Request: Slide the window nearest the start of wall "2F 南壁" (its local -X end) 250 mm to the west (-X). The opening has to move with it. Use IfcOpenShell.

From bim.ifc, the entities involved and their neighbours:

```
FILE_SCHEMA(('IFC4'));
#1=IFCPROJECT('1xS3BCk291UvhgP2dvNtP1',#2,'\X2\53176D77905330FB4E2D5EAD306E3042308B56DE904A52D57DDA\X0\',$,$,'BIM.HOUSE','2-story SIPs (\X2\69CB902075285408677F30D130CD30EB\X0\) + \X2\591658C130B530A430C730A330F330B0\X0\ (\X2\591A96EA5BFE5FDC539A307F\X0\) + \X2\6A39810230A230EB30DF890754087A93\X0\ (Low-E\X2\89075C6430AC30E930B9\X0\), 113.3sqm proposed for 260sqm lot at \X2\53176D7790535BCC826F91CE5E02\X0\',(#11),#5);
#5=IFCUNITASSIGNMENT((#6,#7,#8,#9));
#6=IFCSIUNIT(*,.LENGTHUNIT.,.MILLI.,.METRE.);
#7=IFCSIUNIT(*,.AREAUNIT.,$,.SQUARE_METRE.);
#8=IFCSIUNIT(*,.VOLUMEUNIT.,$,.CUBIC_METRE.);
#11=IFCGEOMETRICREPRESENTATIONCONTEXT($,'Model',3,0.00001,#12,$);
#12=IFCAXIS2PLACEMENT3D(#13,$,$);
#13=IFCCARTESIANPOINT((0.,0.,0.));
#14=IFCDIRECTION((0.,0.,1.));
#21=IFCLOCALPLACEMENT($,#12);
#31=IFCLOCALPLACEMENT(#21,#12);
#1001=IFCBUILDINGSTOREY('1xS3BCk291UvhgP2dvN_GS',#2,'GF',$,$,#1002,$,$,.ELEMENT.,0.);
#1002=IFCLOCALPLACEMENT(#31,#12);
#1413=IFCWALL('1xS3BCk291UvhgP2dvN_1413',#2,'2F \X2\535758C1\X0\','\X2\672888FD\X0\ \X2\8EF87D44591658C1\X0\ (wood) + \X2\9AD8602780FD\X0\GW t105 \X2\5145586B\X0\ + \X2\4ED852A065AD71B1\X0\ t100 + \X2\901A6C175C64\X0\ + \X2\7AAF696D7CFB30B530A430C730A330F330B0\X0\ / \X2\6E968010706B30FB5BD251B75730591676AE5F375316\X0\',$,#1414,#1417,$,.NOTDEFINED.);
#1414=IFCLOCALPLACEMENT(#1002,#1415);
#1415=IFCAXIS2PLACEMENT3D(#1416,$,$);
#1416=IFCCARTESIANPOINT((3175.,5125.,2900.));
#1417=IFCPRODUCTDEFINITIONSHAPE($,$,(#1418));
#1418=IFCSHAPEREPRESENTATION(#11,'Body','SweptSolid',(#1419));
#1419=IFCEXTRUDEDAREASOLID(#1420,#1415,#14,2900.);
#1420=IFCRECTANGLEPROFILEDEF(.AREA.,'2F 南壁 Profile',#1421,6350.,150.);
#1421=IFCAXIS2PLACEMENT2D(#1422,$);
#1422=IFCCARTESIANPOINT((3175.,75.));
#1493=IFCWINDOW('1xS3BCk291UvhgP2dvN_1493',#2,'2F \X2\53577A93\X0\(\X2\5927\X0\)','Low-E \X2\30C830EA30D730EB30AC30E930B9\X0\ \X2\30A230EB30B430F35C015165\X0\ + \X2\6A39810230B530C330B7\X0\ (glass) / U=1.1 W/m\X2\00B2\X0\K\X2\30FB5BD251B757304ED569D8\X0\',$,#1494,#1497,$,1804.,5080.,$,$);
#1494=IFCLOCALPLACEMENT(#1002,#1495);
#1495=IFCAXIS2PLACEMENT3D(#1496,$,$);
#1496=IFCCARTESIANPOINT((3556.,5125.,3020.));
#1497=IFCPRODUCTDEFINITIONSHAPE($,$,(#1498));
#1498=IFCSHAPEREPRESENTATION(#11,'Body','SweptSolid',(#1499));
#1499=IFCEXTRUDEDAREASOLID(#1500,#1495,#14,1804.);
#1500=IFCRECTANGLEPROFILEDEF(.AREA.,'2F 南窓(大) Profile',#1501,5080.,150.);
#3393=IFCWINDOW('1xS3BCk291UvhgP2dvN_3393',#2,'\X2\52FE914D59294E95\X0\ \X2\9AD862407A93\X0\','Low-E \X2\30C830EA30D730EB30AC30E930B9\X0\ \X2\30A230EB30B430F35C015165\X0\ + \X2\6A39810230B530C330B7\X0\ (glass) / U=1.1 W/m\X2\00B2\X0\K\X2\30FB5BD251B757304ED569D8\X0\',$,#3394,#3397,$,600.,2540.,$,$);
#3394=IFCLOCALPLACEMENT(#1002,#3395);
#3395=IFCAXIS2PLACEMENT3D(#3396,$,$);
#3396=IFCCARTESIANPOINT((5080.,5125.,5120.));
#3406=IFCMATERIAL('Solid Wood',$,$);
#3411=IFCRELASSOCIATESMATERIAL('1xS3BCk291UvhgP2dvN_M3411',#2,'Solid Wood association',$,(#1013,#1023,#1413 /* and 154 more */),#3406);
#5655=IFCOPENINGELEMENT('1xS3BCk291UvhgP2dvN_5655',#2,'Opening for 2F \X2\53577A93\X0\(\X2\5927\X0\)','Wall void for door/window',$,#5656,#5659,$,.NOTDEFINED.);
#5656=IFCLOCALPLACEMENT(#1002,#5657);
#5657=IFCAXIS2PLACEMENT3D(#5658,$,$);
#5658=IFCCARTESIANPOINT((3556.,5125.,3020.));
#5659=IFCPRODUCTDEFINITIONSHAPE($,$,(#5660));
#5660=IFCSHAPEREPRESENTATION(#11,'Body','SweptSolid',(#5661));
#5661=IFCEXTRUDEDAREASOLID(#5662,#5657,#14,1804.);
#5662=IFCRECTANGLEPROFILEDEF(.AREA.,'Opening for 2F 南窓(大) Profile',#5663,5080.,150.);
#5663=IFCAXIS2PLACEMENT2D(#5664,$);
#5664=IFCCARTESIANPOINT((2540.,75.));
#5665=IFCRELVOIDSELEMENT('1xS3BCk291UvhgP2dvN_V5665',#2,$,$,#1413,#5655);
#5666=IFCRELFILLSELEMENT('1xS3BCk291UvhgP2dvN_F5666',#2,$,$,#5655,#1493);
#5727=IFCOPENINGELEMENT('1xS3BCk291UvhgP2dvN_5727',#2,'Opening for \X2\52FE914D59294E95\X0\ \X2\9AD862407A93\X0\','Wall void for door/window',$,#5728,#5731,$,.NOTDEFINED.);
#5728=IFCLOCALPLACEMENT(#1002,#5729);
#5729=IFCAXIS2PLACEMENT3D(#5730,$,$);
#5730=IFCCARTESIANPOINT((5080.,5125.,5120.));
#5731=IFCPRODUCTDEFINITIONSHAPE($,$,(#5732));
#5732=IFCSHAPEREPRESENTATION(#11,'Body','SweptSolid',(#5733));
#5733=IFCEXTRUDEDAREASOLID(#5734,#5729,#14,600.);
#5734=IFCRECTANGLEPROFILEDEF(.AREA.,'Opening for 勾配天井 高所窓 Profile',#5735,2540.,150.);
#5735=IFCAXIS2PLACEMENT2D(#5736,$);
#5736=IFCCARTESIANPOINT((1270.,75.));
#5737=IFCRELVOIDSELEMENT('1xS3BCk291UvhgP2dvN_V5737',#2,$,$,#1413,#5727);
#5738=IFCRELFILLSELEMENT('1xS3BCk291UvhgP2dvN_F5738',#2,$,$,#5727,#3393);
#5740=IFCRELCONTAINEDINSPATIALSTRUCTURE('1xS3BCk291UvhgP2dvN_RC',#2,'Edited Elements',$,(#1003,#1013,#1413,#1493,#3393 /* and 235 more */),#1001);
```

```python
import ifcopenshell
import ifcopenshell.api.geometry
import ifcopenshell.util.placement
import ifcopenshell.util.unit

model = ifcopenshell.open("bim.ifc")
unit_scale = ifcopenshell.util.unit.calculate_unit_scale(model)

window = model.by_guid("1xS3BCk291UvhgP2dvN_1493")
opening = window.FillsVoids[0].RelatingOpeningElement
wall = opening.VoidsElements[0].RelatingBuildingElement

wall_matrix = ifcopenshell.util.placement.get_local_placement(wall.ObjectPlacement)
shift = wall_matrix[:3, 0] * -0.25 / unit_scale
before = ifcopenshell.util.placement.get_local_placement(window.ObjectPlacement)[:3, 3].copy()

# The window is not placed relative to its opening, so move both.
for product in (opening, window):
    matrix = ifcopenshell.util.placement.get_local_placement(product.ObjectPlacement)
    matrix[:3, 3] += shift
    ifcopenshell.api.geometry.edit_object_placement(model, product=product, matrix=matrix, is_si=False)

after = ifcopenshell.util.placement.get_local_placement(window.ObjectPlacement)[:3, 3]
print("window moved by", (after - before).round(3) + 0.0)

model.write("bim-out.ifc")
```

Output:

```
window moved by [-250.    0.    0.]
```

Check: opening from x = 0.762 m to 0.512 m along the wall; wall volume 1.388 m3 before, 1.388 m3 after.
